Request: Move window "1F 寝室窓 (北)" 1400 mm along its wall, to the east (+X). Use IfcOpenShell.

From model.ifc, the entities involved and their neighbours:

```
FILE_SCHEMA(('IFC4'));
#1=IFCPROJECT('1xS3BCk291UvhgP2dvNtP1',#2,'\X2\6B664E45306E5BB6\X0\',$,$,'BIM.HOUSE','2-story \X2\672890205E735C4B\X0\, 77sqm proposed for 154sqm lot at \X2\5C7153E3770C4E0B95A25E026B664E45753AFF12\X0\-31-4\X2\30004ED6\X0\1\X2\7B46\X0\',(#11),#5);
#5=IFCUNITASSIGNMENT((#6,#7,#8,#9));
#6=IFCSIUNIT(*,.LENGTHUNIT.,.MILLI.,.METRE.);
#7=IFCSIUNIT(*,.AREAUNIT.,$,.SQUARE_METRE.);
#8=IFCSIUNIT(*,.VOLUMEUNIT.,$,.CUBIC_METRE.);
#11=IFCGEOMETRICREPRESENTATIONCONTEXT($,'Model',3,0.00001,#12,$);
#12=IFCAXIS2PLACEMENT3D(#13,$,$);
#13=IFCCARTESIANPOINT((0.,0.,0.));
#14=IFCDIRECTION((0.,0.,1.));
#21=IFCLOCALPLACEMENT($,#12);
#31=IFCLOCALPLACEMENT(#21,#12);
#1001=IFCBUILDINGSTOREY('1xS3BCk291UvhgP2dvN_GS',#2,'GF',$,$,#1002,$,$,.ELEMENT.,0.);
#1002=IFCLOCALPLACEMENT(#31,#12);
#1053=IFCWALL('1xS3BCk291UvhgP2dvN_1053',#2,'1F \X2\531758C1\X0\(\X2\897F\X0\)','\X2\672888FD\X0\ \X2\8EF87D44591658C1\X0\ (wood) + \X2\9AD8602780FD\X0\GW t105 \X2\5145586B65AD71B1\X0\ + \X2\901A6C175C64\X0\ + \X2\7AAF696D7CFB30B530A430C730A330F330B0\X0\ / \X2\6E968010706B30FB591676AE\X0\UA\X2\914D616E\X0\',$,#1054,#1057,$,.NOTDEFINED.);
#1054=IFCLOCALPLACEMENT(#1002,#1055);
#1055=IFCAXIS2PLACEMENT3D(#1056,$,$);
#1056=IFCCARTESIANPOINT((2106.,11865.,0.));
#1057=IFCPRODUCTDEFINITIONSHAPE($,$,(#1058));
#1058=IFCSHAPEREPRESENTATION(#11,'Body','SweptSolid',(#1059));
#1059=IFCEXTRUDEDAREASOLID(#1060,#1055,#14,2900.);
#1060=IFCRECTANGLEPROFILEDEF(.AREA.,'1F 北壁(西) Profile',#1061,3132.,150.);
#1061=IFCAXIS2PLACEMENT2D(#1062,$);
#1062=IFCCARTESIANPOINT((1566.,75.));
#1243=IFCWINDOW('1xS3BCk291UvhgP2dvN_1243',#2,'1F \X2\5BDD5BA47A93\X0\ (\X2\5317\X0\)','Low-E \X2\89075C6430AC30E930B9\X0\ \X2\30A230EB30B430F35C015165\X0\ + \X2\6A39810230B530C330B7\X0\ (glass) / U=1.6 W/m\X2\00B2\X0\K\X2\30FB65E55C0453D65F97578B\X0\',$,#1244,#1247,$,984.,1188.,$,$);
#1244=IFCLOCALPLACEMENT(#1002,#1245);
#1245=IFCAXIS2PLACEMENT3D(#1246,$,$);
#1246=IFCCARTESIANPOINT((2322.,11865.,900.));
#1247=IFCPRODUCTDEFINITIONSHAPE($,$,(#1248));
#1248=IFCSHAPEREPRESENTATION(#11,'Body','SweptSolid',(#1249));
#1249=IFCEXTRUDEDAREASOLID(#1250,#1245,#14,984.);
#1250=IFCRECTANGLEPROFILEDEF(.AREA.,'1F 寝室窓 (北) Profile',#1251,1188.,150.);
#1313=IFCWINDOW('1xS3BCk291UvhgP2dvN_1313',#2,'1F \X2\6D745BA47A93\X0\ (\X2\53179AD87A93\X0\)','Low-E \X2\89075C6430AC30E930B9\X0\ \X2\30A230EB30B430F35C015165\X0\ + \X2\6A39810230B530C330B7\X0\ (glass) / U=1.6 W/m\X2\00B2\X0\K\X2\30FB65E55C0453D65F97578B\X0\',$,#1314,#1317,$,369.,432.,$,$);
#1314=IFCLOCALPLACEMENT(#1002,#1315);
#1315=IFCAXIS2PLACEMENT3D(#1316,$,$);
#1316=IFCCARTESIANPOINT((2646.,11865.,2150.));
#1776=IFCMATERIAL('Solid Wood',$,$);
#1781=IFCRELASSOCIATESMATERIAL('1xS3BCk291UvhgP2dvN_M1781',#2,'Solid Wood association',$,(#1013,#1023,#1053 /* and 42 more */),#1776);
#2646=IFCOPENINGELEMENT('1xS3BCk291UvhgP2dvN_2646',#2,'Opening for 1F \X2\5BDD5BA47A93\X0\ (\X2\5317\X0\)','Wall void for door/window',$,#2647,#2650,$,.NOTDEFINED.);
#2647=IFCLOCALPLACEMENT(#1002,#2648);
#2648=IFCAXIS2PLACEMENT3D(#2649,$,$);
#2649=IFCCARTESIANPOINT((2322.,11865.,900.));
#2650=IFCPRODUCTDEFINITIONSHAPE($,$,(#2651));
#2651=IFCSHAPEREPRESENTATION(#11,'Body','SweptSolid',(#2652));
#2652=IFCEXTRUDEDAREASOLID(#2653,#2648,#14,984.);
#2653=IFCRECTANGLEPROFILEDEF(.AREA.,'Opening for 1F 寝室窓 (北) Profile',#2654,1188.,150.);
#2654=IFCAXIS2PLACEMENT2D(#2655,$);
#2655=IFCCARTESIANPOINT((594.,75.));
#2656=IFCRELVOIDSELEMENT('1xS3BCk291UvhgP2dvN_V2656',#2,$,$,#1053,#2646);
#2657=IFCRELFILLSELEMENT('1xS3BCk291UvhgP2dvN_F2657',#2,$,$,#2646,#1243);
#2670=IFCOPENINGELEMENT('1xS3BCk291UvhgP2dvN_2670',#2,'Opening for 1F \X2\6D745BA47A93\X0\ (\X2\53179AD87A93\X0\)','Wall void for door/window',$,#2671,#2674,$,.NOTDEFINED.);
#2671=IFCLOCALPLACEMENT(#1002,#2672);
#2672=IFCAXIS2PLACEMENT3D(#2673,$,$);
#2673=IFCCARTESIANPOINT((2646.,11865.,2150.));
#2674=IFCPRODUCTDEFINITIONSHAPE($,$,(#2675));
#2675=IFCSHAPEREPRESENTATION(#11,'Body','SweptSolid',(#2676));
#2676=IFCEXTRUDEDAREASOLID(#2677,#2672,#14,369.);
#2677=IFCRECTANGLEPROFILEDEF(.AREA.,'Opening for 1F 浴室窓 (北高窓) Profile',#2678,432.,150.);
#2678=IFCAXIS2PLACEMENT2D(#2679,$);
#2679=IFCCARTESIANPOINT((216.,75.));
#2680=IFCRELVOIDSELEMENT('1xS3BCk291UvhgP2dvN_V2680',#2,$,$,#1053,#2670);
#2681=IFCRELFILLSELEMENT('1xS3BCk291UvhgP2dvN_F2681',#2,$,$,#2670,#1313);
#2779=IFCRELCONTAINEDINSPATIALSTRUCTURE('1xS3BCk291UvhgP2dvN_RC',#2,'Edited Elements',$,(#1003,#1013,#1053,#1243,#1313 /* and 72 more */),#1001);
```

```python
import ifcopenshell
import ifcopenshell.api.geometry
import ifcopenshell.util.placement
import ifcopenshell.util.unit

model = ifcopenshell.open("model.ifc")
unit_scale = ifcopenshell.util.unit.calculate_unit_scale(model)

window = model.by_guid("1xS3BCk291UvhgP2dvN_1243")
opening = window.FillsVoids[0].RelatingOpeningElement
wall = opening.VoidsElements[0].RelatingBuildingElement

wall_matrix = ifcopenshell.util.placement.get_local_placement(wall.ObjectPlacement)
shift = wall_matrix[:3, 0] * 1.4 / unit_scale
before = ifcopenshell.util.placement.get_local_placement(window.ObjectPlacement)[:3, 3].copy()

# The window is not placed relative to its opening, so move both.
for product in (opening, window):
    matrix = ifcopenshell.util.placement.get_local_placement(product.ObjectPlacement)
    matrix[:3, 3] += shift
    ifcopenshell.api.geometry.edit_object_placement(model, product=product, matrix=matrix, is_si=False)

after = ifcopenshell.util.placement.get_local_placement(window.ObjectPlacement)[:3, 3]
print("window moved by", (after - before).round(3) + 0.0)

model.write("model_updated.ifc")
```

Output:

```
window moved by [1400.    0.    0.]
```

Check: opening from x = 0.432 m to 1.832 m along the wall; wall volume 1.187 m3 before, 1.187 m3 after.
